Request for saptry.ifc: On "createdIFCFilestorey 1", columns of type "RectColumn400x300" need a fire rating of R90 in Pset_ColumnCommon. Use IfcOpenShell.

First a look at what the model holds.

```python
import ifcopenshell
import ifcopenshell.util.element

model = ifcopenshell.open("saptry.ifc")
print(model.schema)
storey = next(s for s in model.by_type("IfcBuildingStorey") if s.Name == "createdIFCFilestorey 1")
columns = [e for e in ifcopenshell.util.element.get_decomposition(storey) if e.is_a("IfcColumn")]
seen = {}
for e in columns:
    element_type = ifcopenshell.util.element.get_type(e)
    key = (element_type.Name if element_type != e and element_type else None, ifcopenshell.util.element.get_pset(e, "Pset_ColumnCommon", "FireRating"))
    seen[key] = seen.get(key, 0) + 1
for (name, value), count in sorted(seen.items(), key=str):
    print(count, "x", name, "|", value)
```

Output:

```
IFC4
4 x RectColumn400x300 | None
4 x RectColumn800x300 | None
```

```python
import ifcopenshell
import ifcopenshell.api.pset
import ifcopenshell.util.element

model = ifcopenshell.open("saptry.ifc")

storey = next(s for s in model.by_type("IfcBuildingStorey") if s.Name == "createdIFCFilestorey 1")
columns = [e for e in ifcopenshell.util.element.get_decomposition(storey) if e.is_a("IfcColumn")]

count = 0
for e in columns:
    element_type = ifcopenshell.util.element.get_type(e)
    if element_type in (None, e) or element_type.Name != "RectColumn400x300":
        continue
    # add_pset returns the element's existing set when there is one.
    pset = ifcopenshell.api.pset.add_pset(model, product=e, name="Pset_ColumnCommon")
    ifcopenshell.api.pset.edit_pset(model, pset=pset, properties={"FireRating": "R90"})
    count += 1

print(count, "columns updated")

model.write("saptry-out.ifc")
```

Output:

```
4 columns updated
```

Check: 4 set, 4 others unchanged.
